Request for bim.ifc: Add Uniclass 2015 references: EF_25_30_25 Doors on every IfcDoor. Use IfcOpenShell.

First a look at what the model holds.

```python
import ifcopenshell

model = ifcopenshell.open("bim.ifc")
print(model.schema)
print("classifications:", [c.Name for c in model.by_type("IfcClassification")])
for ifc_class in ("IfcDoor", "IfcRoof", "IfcStair", "IfcWall", "IfcWindow"):
    print(ifc_class, len(model.by_type(ifc_class)))
```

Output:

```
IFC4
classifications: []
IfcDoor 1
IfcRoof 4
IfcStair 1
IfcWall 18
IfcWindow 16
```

```python
import ifcopenshell
import ifcopenshell.api.classification

model = ifcopenshell.open("bim.ifc")

system = ifcopenshell.api.classification.add_classification(model, classification="Uniclass 2015")

codes = {
    "IfcDoor": ("EF_25_30_25", "Doors"),
}
for ifc_class, (code, name) in codes.items():
    products = model.by_type(ifc_class)
    ifcopenshell.api.classification.add_reference(
        model, products=products, classification=system, identification=code, name=name
    )
    print(code, len(products))

model.write("bim_v2.ifc")
```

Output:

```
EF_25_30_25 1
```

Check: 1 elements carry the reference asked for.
